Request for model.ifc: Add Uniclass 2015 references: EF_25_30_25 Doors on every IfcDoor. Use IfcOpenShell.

First a look at what the model holds.

```python
import ifcopenshell

model = ifcopenshell.open("model.ifc")
print(model.schema)
print("classifications:", [c.Name for c in model.by_type("IfcClassification")])
for ifc_class in ("IfcDoor", "IfcRoof", "IfcStair", "IfcWall", "IfcWindow"):
    print(ifc_class, len(model.by_type(ifc_class)))
```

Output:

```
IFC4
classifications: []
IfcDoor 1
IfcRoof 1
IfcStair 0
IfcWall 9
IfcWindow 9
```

```python
import ifcopenshell
import ifcopenshell.api.classification

model = ifcopenshell.open("model.ifc")

system = ifcopenshell.api.classification.add_classification(model, classification="Uniclass 2015")

codes = {
    "IfcDoor": ("EF_25_30_25", "Doors"),
}
for ifc_class, (code, name) in codes.items():
    products = model.by_type(ifc_class)
    ifcopenshell.api.classification.add_reference(
        model, products=products, classification=system, identification=code, name=name
    )
    print(code, len(products))

model.write("model_v2.ifc")
```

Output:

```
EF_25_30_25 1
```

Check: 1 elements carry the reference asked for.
